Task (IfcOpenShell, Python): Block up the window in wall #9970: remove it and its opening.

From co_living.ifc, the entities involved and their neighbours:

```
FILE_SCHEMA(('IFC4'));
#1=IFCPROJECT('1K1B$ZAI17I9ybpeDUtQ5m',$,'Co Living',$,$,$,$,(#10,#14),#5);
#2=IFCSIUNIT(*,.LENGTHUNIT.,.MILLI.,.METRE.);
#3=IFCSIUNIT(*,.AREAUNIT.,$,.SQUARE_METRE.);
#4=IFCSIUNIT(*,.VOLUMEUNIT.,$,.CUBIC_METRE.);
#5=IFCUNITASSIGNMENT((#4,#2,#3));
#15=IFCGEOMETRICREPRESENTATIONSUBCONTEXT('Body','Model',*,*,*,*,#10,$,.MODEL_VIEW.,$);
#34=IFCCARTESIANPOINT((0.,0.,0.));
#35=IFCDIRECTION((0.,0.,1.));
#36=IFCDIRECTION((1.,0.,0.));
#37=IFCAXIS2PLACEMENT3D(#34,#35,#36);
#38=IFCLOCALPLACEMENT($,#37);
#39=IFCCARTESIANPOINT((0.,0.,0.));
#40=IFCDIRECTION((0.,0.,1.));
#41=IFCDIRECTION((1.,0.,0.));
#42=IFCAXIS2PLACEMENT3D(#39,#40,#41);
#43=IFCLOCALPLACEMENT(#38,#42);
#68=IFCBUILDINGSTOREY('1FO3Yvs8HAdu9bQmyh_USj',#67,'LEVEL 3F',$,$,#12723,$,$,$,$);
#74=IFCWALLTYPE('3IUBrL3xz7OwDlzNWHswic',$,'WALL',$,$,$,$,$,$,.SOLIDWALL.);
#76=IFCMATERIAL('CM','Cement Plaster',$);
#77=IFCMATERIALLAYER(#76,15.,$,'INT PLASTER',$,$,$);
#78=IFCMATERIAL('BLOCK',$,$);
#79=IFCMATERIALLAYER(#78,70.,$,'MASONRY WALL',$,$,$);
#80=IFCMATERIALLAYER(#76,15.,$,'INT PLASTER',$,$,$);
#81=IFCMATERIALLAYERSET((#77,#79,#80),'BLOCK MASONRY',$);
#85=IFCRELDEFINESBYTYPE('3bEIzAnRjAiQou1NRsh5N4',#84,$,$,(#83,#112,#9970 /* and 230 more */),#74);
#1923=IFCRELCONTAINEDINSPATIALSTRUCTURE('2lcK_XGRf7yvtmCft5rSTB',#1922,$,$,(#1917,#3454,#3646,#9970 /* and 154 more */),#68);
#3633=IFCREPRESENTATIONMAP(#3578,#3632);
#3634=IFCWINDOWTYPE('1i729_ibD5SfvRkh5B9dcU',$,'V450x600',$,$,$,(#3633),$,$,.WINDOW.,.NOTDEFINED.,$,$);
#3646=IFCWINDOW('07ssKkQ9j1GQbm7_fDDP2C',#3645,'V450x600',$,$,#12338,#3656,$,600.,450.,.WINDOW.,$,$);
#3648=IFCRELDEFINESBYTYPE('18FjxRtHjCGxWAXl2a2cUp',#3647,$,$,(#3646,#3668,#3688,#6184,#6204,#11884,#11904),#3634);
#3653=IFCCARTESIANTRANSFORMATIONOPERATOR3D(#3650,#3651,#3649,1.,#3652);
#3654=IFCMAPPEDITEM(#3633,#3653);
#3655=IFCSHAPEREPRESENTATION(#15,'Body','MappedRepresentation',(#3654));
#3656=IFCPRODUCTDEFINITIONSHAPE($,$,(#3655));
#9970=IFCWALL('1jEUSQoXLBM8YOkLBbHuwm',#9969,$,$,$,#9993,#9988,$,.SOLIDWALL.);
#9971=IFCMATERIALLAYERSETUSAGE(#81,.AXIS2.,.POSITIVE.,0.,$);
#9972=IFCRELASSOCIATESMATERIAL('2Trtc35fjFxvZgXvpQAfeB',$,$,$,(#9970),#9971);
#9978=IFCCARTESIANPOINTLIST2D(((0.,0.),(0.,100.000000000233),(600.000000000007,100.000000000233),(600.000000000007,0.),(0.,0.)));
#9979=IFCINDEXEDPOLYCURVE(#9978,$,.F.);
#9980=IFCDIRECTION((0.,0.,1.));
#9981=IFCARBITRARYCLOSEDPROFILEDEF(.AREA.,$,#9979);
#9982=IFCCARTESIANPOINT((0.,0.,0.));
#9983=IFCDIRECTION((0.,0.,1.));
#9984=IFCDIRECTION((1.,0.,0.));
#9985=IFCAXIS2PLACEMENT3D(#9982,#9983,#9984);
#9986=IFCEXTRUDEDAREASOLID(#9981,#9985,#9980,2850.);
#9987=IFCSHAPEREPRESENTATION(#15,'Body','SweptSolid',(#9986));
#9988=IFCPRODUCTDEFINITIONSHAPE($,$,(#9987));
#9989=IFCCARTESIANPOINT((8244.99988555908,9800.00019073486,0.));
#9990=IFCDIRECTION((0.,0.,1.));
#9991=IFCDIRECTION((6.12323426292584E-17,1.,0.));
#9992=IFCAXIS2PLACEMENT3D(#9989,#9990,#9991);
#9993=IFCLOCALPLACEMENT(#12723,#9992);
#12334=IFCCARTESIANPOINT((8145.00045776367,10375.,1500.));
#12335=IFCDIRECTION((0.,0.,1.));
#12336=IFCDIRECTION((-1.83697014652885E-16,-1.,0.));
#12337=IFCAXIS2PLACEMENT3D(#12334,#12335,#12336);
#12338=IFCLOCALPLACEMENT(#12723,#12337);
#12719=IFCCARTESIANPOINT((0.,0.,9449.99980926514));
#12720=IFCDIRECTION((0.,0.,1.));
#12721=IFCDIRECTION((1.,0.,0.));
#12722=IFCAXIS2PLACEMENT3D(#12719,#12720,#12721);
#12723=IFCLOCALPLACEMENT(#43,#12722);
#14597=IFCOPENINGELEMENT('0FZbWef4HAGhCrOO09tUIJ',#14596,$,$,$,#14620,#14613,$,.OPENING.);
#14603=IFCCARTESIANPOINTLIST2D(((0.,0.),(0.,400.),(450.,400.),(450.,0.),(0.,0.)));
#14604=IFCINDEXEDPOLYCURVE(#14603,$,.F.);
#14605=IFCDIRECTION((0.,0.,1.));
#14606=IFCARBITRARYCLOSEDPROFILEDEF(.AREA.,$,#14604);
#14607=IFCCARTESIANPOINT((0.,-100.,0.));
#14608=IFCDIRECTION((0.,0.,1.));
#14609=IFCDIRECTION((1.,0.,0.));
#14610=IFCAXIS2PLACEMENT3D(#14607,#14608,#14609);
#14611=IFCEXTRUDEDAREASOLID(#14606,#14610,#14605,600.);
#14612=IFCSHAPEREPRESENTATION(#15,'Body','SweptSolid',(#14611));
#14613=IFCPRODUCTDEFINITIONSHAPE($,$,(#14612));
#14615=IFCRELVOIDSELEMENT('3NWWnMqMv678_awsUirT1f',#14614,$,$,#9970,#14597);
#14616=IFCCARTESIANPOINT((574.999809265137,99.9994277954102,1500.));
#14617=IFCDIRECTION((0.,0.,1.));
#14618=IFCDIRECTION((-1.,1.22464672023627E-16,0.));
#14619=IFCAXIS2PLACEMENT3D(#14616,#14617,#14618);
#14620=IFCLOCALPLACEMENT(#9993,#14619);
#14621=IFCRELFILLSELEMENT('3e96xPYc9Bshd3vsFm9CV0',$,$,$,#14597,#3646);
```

```python
import ifcopenshell
import ifcopenshell.api.feature
import ifcopenshell.api.root
import ifcopenshell.geom
import ifcopenshell.util.shape

model = ifcopenshell.open("co_living.ifc")
settings = ifcopenshell.geom.settings()


def volume(element):
    """Net volume in cubic metres, openings subtracted."""
    shape = ifcopenshell.geom.create_shape(settings, element)
    return ifcopenshell.util.shape.get_volume(shape.geometry)


window = model.by_guid("07ssKkQ9j1GQbm7_fDDP2C")
opening = window.FillsVoids[0].RelatingOpeningElement
wall = opening.VoidsElements[0].RelatingBuildingElement
before = volume(wall)

ifcopenshell.api.root.remove_product(model, product=window)
ifcopenshell.api.feature.remove_feature(model, feature=opening)

after = volume(wall)

print(f"wall volume {before:.3f} -> {after:.3f} m3")

model.write("co_living-out.ifc")
```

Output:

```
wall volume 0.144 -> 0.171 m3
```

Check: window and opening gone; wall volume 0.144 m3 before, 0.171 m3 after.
